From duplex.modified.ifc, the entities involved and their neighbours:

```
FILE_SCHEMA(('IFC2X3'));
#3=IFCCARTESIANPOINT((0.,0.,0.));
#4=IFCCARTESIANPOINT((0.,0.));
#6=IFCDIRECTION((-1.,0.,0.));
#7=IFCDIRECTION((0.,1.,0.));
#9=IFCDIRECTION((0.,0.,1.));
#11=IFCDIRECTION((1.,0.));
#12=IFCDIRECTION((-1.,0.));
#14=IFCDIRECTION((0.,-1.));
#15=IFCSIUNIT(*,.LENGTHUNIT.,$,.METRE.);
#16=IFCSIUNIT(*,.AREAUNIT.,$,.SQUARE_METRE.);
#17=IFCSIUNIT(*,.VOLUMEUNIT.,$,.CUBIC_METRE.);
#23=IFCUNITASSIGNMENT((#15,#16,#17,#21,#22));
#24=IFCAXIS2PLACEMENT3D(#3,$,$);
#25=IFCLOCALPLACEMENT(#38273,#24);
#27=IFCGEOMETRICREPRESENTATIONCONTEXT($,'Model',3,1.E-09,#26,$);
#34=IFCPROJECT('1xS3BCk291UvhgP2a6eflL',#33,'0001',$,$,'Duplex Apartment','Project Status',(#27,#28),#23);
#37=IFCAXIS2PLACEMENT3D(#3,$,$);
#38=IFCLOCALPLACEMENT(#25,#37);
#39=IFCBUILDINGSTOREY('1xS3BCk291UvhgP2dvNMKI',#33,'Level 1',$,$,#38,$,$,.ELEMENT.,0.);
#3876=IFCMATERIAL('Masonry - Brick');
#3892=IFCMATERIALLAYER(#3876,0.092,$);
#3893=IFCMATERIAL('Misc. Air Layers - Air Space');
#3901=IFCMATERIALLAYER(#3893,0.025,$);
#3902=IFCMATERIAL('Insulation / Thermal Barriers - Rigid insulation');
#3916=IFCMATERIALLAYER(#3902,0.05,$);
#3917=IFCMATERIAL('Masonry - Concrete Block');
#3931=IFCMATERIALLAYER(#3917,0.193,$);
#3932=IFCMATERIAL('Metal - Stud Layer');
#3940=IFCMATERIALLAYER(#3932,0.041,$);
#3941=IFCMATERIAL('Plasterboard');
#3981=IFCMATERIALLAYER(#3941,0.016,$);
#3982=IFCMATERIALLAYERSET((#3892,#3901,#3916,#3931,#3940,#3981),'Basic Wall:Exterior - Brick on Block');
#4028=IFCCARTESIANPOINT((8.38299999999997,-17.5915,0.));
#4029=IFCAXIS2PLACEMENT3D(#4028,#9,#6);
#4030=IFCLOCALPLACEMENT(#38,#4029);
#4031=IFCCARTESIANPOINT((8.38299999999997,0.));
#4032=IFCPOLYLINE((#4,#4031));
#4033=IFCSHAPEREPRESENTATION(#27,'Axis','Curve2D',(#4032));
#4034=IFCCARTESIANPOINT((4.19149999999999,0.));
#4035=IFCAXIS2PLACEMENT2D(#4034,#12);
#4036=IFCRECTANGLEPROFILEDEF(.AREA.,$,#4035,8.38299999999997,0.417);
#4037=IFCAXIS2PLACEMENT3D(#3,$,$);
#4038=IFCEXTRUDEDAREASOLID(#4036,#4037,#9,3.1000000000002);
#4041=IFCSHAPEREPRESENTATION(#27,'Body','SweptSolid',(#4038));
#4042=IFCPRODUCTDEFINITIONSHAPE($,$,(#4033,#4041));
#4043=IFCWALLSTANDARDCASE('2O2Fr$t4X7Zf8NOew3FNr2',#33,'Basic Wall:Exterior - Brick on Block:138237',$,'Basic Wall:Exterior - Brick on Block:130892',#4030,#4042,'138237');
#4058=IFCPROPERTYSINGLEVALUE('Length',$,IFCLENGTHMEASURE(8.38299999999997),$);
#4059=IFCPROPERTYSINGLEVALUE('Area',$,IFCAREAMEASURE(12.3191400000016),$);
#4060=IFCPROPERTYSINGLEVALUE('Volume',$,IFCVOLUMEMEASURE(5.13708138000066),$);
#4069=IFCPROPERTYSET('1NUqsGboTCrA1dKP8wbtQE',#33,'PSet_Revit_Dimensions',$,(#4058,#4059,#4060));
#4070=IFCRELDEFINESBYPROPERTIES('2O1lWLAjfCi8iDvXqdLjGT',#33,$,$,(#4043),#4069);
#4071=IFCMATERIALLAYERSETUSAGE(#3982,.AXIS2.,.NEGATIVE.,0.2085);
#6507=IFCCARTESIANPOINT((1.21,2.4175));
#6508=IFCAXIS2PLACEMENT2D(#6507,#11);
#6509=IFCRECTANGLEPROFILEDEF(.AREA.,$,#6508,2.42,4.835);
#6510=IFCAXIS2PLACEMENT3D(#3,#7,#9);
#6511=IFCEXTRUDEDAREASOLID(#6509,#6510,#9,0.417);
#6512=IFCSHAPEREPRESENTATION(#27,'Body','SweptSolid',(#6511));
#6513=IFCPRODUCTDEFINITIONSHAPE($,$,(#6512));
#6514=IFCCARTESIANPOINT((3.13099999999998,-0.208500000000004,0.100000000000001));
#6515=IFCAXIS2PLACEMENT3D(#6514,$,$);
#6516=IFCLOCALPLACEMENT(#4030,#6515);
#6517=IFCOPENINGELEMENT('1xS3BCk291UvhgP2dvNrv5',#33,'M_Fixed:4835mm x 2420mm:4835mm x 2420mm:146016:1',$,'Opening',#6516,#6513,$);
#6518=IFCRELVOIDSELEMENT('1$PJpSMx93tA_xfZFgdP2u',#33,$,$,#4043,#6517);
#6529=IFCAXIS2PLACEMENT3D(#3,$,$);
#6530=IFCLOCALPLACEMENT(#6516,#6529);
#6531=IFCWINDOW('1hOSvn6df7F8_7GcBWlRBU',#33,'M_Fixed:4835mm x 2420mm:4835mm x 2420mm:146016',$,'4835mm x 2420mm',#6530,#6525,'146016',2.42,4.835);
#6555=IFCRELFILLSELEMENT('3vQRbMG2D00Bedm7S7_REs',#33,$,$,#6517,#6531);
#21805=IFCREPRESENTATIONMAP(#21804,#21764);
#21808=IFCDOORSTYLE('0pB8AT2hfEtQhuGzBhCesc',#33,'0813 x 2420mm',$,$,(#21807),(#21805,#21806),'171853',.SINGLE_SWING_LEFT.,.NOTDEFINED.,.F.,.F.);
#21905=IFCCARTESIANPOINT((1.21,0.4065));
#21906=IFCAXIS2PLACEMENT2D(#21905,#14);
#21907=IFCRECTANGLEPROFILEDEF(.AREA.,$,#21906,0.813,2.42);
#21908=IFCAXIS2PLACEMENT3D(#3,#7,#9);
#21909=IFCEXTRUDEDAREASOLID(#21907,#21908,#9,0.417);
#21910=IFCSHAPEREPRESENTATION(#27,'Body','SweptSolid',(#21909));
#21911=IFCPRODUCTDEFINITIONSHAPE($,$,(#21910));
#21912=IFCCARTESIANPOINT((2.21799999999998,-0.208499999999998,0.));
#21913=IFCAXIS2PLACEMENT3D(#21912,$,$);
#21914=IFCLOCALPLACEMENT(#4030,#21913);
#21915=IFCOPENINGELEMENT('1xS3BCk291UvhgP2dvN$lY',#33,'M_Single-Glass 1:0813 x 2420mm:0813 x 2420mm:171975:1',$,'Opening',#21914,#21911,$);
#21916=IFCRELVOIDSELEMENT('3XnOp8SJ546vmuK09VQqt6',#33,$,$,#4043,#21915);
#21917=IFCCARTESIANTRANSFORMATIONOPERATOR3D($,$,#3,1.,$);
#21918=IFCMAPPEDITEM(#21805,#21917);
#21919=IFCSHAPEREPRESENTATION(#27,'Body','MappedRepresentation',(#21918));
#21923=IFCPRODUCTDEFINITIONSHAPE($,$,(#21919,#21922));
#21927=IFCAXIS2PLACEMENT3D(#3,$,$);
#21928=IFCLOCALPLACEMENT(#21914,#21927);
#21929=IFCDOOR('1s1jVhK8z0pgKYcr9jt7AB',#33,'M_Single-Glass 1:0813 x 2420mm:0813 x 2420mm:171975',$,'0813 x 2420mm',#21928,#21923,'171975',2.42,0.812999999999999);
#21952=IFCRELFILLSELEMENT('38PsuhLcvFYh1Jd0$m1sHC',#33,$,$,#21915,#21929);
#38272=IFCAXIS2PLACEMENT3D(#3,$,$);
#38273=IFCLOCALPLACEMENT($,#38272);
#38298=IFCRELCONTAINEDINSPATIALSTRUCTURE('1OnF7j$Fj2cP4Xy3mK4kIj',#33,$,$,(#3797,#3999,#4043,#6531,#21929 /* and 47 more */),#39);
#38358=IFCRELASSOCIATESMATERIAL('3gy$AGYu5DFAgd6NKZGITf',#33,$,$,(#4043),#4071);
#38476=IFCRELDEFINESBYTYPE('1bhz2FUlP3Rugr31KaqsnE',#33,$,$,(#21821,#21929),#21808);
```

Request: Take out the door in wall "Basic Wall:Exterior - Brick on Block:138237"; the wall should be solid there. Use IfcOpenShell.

```python
import ifcopenshell
import ifcopenshell.api.feature
import ifcopenshell.api.pset
import ifcopenshell.api.root
import ifcopenshell.geom
import ifcopenshell.util.element
import ifcopenshell.util.shape
import ifcopenshell.util.unit

model = ifcopenshell.open("duplex.modified.ifc")
area_scale = ifcopenshell.util.unit.calculate_unit_scale(model, "AREAUNIT")
volume_scale = ifcopenshell.util.unit.calculate_unit_scale(model, "VOLUMEUNIT")
settings = ifcopenshell.geom.settings()


def volume(element):
    """Net volume in cubic metres, openings subtracted."""
    shape = ifcopenshell.geom.create_shape(settings, element)
    return ifcopenshell.util.shape.get_volume(shape.geometry)


door = model.by_guid("1s1jVhK8z0pgKYcr9jt7AB")
opening = door.FillsVoids[0].RelatingOpeningElement
wall = opening.VoidsElements[0].RelatingBuildingElement
before = volume(wall)

ifcopenshell.api.root.remove_product(model, product=door)
ifcopenshell.api.feature.remove_feature(model, feature=opening)

after = volume(wall)
thickness = 0.417  # wall thickness in metres

# Update the wall's stored quantities.
pset = model.by_id(ifcopenshell.util.element.get_pset(wall, "PSet_Revit_Dimensions", should_inherit=False)["id"])
ifcopenshell.api.pset.edit_pset(model, pset=pset, properties={
    "Area": model.create_entity("IfcAreaMeasure", after / thickness / area_scale),
    "Volume": model.create_entity("IfcVolumeMeasure", after / volume_scale),
})

print(f"wall volume {before:.3f} -> {after:.3f} m3")

model.write("duplex.modified_updated.ifc")
```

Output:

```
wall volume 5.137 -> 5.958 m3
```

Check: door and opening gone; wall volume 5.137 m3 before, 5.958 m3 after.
